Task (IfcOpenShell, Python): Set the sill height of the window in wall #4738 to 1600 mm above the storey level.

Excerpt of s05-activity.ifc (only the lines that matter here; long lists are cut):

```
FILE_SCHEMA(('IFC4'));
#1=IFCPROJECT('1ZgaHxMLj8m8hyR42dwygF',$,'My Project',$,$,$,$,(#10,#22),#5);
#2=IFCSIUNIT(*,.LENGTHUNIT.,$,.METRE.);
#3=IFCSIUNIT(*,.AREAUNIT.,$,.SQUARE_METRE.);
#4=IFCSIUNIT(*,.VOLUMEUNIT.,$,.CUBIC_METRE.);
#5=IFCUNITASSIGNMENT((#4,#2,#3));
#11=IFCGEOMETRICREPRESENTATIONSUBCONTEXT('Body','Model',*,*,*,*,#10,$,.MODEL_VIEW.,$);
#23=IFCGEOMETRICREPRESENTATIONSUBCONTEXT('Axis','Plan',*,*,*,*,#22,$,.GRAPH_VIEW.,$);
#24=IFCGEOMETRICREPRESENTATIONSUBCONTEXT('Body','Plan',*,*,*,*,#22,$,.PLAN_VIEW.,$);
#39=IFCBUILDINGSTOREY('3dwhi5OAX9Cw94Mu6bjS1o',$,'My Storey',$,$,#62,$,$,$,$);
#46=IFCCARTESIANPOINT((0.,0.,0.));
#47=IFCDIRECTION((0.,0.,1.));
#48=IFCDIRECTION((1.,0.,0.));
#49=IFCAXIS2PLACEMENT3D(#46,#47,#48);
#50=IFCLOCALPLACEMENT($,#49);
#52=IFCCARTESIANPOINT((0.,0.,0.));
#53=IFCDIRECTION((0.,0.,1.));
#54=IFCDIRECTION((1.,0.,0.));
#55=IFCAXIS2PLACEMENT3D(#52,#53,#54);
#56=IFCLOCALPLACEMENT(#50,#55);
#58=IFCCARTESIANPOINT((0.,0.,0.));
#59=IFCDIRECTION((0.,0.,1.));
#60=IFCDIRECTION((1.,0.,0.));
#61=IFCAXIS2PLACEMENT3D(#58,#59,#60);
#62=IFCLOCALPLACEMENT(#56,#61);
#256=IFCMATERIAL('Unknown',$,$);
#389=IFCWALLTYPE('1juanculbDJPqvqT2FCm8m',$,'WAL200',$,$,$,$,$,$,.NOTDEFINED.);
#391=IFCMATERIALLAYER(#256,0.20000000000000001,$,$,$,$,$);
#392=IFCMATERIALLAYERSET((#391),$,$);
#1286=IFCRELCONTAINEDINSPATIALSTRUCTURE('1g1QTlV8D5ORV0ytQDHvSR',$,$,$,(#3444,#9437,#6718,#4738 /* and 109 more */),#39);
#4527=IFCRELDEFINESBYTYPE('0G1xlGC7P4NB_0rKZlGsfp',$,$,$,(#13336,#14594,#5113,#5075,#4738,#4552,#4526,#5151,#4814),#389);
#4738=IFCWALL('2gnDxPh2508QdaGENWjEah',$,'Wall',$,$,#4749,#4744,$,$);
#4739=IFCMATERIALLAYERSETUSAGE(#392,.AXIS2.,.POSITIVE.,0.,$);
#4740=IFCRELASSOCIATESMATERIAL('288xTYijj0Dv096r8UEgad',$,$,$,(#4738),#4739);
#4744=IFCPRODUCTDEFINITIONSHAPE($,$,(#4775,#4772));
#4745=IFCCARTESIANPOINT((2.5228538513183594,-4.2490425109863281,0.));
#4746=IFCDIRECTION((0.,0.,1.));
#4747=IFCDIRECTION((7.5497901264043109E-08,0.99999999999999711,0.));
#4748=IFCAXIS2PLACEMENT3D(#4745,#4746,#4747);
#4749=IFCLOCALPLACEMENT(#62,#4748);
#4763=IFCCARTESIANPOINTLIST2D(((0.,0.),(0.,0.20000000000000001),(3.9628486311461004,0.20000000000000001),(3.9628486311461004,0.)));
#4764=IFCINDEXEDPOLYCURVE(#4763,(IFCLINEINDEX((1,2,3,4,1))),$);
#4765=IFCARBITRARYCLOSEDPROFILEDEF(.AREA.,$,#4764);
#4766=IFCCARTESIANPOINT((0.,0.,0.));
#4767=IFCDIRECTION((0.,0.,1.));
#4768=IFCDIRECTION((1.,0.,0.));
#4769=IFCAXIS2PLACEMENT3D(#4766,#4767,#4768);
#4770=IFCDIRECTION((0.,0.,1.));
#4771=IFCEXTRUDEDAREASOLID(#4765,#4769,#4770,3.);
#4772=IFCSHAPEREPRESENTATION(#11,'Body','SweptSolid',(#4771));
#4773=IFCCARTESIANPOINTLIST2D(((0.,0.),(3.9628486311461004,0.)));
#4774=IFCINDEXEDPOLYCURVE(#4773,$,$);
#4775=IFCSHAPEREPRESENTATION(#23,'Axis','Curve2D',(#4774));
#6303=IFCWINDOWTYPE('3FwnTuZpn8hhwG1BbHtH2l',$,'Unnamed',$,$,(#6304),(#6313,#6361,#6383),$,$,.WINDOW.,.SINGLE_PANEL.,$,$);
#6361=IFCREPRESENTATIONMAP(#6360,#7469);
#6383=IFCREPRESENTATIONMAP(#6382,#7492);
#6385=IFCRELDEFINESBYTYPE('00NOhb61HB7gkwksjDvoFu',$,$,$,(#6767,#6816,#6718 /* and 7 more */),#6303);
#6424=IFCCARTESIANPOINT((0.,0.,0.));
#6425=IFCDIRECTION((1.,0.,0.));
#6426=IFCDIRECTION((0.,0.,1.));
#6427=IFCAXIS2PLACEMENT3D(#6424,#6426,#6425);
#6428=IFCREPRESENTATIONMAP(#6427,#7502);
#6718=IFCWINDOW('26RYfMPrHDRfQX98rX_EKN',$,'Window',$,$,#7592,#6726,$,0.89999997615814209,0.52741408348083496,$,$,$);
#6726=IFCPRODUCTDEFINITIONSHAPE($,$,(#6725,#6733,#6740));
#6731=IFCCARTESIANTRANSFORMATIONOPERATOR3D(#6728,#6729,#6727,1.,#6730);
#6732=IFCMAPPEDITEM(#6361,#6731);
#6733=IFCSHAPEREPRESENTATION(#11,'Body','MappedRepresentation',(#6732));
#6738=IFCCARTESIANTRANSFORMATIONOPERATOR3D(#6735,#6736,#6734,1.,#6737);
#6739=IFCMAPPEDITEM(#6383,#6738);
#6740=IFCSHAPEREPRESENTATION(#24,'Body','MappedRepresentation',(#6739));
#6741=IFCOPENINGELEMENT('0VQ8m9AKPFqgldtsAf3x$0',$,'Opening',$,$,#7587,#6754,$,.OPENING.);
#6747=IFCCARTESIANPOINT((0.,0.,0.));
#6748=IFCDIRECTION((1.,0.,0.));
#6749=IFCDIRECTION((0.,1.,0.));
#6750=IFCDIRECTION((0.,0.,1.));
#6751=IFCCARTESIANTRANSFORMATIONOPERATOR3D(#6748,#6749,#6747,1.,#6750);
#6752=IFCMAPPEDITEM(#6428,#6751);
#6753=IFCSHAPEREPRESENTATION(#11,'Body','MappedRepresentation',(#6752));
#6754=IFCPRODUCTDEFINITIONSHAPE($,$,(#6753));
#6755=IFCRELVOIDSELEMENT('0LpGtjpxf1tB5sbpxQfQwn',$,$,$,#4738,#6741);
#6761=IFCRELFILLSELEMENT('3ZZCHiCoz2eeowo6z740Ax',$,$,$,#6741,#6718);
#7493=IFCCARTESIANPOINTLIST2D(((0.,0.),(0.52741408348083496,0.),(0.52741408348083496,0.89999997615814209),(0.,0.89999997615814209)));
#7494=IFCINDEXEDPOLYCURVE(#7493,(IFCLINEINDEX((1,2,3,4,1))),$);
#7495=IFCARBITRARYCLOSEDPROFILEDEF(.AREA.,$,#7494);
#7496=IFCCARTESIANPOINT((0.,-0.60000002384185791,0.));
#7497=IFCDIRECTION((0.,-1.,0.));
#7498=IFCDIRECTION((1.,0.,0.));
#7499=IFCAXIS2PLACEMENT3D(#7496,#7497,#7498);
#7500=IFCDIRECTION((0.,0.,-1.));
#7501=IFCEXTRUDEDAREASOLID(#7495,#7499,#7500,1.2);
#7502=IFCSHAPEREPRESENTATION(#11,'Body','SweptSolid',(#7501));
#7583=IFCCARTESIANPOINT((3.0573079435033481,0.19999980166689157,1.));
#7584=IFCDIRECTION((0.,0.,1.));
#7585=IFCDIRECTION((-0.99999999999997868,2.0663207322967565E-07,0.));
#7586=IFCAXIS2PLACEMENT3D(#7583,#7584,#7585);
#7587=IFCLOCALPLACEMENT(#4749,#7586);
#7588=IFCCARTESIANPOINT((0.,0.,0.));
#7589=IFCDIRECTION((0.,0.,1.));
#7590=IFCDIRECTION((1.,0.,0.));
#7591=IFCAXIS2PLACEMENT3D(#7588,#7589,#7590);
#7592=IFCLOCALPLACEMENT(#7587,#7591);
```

```python
import numpy as np
import ifcopenshell
import ifcopenshell.api.geometry
import ifcopenshell.geom
import ifcopenshell.util.element
import ifcopenshell.util.placement
import ifcopenshell.util.shape
import ifcopenshell.util.unit

model = ifcopenshell.open("s05-activity.ifc")
unit_scale = ifcopenshell.util.unit.calculate_unit_scale(model)

window = model.by_id(6718)
opening = window.FillsVoids[0].RelatingOpeningElement
storey = ifcopenshell.util.element.get_container(window, ifc_class="IfcBuildingStorey")
level = ifcopenshell.util.placement.get_local_placement(storey.ObjectPlacement)[2, 3]

# The opening's origin need not be at the sill, so measure its lowest point.
shape = ifcopenshell.geom.create_shape(ifcopenshell.geom.settings(), opening)
bottom = ifcopenshell.util.shape.get_shape_bottom_elevation(shape, shape.geometry) / unit_scale
dz = level + 1.6 / unit_scale - bottom

shift = np.array([0.0, 0.0, dz])
# The window is placed relative to its opening, so it follows when the opening moves.
matrix = ifcopenshell.util.placement.get_local_placement(opening.ObjectPlacement)
matrix[:3, 3] += shift
ifcopenshell.api.geometry.edit_object_placement(
    model, product=opening, matrix=matrix, is_si=False, should_transform_children=True
)

print(f"moved by {dz * unit_scale:+.3f} m")

model.write("s05-activity_rev.ifc")
```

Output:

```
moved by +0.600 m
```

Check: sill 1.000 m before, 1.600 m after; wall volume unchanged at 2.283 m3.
